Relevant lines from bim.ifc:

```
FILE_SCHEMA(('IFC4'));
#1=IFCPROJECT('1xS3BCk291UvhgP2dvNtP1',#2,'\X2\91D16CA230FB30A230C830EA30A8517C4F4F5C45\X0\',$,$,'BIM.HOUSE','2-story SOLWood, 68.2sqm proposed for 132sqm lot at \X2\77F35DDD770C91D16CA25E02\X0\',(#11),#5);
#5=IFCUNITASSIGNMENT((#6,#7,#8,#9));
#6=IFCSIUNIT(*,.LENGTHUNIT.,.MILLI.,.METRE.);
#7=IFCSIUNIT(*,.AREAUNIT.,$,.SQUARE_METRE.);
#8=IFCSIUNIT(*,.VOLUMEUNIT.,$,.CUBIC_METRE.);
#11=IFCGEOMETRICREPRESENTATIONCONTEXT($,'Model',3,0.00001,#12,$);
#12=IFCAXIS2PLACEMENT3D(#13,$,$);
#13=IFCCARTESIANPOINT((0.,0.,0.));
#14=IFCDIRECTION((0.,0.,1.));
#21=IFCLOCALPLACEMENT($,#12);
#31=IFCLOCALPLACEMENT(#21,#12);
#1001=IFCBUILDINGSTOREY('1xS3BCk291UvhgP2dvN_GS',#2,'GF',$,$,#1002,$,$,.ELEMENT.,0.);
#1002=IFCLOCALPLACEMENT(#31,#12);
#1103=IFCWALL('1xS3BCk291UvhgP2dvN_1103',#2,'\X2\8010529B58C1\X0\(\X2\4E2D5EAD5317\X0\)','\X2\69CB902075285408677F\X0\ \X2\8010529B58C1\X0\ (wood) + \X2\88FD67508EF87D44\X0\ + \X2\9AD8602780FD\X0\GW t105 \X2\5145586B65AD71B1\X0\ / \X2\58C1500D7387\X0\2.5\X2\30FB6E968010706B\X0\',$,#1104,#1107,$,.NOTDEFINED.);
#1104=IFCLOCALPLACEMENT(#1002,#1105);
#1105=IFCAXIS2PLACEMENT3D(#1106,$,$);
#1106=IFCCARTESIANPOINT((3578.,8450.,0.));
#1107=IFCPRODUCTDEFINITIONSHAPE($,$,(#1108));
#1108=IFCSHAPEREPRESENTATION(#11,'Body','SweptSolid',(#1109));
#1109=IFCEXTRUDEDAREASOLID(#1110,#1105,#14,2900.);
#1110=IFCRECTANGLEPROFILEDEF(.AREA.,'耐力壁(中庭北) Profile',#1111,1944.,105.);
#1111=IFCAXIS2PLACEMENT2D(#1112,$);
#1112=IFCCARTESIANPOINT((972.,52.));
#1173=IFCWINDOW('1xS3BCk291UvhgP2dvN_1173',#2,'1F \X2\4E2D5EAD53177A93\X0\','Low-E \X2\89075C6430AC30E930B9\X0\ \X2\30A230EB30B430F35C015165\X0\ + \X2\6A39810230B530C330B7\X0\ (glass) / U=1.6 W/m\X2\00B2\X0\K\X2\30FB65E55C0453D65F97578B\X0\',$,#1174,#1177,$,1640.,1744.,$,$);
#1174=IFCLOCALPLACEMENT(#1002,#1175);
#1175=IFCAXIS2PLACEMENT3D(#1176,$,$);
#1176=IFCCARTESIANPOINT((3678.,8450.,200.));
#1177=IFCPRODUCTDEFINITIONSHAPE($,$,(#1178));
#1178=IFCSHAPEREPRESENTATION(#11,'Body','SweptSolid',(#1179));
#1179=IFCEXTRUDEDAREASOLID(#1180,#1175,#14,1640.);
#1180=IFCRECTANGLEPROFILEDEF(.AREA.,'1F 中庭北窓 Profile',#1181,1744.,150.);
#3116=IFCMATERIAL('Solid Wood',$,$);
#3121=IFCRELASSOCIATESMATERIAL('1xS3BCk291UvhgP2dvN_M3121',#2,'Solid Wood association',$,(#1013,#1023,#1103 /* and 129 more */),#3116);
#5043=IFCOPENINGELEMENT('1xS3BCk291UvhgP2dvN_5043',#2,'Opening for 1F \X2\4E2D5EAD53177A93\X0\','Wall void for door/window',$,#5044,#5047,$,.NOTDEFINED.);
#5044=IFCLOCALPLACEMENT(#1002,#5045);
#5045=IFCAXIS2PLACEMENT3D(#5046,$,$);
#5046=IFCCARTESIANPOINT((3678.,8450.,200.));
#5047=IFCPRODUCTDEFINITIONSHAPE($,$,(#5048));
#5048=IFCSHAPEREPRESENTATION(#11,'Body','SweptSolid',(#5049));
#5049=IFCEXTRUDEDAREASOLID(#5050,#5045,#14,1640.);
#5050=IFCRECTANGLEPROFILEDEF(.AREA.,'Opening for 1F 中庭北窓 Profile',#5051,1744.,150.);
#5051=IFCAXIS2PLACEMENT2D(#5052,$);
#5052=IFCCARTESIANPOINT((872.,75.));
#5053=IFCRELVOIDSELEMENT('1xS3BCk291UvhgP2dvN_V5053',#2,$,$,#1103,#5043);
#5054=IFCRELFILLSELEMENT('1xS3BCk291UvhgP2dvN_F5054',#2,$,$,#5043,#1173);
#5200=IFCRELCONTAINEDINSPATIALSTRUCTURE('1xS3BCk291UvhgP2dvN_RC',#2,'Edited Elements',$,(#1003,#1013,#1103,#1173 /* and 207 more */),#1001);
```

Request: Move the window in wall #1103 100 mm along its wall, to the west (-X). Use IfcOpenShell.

```python
import ifcopenshell
import ifcopenshell.api.geometry
import ifcopenshell.util.placement
import ifcopenshell.util.unit

model = ifcopenshell.open("bim.ifc")
unit_scale = ifcopenshell.util.unit.calculate_unit_scale(model)

window = model.by_guid("1xS3BCk291UvhgP2dvN_1173")
opening = window.FillsVoids[0].RelatingOpeningElement
wall = opening.VoidsElements[0].RelatingBuildingElement

wall_matrix = ifcopenshell.util.placement.get_local_placement(wall.ObjectPlacement)
shift = wall_matrix[:3, 0] * -0.1 / unit_scale
before = ifcopenshell.util.placement.get_local_placement(window.ObjectPlacement)[:3, 3].copy()

# The window is not placed relative to its opening, so move both.
for product in (opening, window):
    matrix = ifcopenshell.util.placement.get_local_placement(product.ObjectPlacement)
    matrix[:3, 3] += shift
    ifcopenshell.api.geometry.edit_object_placement(model, product=product, matrix=matrix, is_si=False)

after = ifcopenshell.util.placement.get_local_placement(window.ObjectPlacement)[:3, 3]
print("window moved by", (after - before).round(3) + 0.0)

model.write("bim-out.ifc")
```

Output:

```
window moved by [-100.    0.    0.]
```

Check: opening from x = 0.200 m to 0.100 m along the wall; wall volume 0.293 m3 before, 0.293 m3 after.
